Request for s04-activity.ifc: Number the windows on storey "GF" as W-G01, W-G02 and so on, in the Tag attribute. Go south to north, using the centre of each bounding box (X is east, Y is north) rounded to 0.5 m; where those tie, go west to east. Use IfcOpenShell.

First a look at what the model holds.

```python
import ifcopenshell
import ifcopenshell.util.element
import ifcopenshell.util.placement

model = ifcopenshell.open("s04-activity.ifc")
print(model.schema)
storey = next(s for s in model.by_type("IfcBuildingStorey") if s.Name == "GF")
windows = [e for e in ifcopenshell.util.element.get_decomposition(storey) if e.is_a("IfcWindow")]
for e in sorted(windows, key=lambda e: e.id()):
    origin = ifcopenshell.util.placement.get_local_placement(e.ObjectPlacement)[:3, 3]
    print(e.id(), e.Tag, e.Name, origin.round(2) + 0.0, sep=" | ")
```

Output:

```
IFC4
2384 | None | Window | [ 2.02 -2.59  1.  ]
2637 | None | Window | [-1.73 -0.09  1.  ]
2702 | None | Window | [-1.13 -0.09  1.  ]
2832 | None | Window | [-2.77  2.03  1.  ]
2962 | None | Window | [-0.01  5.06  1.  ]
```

```python
import ifcopenshell
import ifcopenshell.geom
import ifcopenshell.util.element
import ifcopenshell.util.shape

model = ifcopenshell.open("s04-activity.ifc")
settings = ifcopenshell.geom.settings()
settings.set("use-world-coords", True)


def centre(element):
    shape = ifcopenshell.geom.create_shape(settings, element)
    return ifcopenshell.util.shape.get_bbox_centroid(shape.geometry)


storey = next(s for s in model.by_type("IfcBuildingStorey") if s.Name == "GF")
windows = [e for e in ifcopenshell.util.element.get_decomposition(storey) if e.is_a("IfcWindow")]

# Insertion points can sit at a corner or the storey origin, so sort by the geometry (in metres).
centres = {e: centre(e) for e in windows}
windows.sort(key=lambda e: (round(centres[e][1] / 0.5), centres[e][0]))

for i, e in enumerate(windows, start=1):
    number = f"W-G{i:02d}"
    e.Tag = number
    print(e.id(), number)

model.write("s04-activity_rev.ifc")
```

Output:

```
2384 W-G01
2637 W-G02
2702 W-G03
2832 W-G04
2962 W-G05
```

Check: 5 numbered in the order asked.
